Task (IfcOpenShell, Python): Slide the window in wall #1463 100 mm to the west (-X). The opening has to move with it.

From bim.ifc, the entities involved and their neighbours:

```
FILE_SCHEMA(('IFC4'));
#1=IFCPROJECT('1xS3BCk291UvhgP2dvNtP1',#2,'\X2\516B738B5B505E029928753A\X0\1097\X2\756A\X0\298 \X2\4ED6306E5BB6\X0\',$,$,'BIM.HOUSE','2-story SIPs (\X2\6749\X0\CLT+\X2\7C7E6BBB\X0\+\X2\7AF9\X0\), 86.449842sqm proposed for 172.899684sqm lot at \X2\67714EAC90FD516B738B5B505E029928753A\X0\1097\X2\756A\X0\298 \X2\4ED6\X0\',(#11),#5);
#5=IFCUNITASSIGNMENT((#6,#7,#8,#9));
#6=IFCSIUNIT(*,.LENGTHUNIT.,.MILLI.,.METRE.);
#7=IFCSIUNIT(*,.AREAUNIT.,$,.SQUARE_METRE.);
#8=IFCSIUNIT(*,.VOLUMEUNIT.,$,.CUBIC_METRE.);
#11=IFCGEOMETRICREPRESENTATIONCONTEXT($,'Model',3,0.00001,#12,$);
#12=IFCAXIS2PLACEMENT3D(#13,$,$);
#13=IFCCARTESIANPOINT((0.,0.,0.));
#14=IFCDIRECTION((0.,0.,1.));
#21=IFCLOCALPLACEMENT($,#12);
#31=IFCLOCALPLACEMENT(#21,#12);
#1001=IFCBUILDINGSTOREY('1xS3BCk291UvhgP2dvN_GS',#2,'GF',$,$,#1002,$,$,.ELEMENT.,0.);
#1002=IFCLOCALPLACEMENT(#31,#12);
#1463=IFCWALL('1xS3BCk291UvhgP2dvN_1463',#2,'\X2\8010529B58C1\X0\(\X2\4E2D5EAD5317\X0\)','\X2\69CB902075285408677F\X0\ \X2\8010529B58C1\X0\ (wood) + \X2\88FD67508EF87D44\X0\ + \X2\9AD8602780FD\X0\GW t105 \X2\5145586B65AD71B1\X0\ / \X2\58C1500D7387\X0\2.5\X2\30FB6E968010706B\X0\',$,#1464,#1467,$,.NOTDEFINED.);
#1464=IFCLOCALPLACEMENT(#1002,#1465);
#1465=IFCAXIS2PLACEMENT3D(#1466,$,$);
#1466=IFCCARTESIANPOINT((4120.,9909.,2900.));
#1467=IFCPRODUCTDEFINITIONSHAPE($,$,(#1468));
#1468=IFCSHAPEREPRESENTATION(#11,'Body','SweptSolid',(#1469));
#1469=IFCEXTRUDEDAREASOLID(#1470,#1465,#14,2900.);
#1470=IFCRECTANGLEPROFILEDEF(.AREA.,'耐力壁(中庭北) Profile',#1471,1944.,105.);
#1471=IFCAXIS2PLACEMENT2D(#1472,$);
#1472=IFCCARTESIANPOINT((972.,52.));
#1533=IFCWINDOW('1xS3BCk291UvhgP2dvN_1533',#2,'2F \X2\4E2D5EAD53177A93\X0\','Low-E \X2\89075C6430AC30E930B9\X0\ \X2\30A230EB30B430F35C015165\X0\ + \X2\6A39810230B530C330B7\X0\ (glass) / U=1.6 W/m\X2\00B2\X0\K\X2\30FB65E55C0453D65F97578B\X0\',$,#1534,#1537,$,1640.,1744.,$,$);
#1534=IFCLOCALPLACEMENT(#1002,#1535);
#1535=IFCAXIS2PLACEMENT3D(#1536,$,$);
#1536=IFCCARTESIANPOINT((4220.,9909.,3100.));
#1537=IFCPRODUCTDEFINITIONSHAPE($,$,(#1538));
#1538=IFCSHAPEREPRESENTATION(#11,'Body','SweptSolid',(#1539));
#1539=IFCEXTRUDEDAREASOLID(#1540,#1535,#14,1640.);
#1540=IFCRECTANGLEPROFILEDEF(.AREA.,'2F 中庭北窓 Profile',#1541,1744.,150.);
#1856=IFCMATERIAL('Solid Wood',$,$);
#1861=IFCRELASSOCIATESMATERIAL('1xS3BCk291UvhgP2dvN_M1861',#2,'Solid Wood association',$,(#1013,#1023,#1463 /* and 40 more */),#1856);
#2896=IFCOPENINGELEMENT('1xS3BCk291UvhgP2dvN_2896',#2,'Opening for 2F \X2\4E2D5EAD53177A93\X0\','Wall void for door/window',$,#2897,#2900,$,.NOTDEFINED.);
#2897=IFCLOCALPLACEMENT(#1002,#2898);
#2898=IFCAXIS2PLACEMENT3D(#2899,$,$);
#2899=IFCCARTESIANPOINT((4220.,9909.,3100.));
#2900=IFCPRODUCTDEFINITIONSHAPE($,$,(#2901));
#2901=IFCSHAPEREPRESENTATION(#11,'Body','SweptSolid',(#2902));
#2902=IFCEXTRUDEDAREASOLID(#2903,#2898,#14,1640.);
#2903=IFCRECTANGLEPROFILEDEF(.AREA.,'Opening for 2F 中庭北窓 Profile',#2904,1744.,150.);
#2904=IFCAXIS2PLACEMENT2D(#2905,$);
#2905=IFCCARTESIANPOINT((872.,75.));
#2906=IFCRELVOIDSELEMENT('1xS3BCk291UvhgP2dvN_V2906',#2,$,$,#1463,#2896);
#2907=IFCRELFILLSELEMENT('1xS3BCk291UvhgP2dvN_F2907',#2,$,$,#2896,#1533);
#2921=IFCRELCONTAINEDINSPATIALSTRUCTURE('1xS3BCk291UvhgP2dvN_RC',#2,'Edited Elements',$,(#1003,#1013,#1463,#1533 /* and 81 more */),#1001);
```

```python
import ifcopenshell
import ifcopenshell.api.geometry
import ifcopenshell.util.placement

model = ifcopenshell.open("bim.ifc")

window = model.by_id(1533)
opening = window.FillsVoids[0].RelatingOpeningElement
wall = opening.VoidsElements[0].RelatingBuildingElement

wall_matrix = ifcopenshell.util.placement.get_local_placement(wall.ObjectPlacement)
shift = wall_matrix[:3, 0] * -100.0
before = ifcopenshell.util.placement.get_local_placement(window.ObjectPlacement)[:3, 3].copy()

# The window is not placed relative to its opening, so move both.
for product in (opening, window):
    matrix = ifcopenshell.util.placement.get_local_placement(product.ObjectPlacement)
    matrix[:3, 3] += shift
    ifcopenshell.api.geometry.edit_object_placement(model, product=product, matrix=matrix, is_si=False)

after = ifcopenshell.util.placement.get_local_placement(window.ObjectPlacement)[:3, 3]
print("window moved by", (after - before).round(3) + 0.0)

model.write("bim-out.ifc")
```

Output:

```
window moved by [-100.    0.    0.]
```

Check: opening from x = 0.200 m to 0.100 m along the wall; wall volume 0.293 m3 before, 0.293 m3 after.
